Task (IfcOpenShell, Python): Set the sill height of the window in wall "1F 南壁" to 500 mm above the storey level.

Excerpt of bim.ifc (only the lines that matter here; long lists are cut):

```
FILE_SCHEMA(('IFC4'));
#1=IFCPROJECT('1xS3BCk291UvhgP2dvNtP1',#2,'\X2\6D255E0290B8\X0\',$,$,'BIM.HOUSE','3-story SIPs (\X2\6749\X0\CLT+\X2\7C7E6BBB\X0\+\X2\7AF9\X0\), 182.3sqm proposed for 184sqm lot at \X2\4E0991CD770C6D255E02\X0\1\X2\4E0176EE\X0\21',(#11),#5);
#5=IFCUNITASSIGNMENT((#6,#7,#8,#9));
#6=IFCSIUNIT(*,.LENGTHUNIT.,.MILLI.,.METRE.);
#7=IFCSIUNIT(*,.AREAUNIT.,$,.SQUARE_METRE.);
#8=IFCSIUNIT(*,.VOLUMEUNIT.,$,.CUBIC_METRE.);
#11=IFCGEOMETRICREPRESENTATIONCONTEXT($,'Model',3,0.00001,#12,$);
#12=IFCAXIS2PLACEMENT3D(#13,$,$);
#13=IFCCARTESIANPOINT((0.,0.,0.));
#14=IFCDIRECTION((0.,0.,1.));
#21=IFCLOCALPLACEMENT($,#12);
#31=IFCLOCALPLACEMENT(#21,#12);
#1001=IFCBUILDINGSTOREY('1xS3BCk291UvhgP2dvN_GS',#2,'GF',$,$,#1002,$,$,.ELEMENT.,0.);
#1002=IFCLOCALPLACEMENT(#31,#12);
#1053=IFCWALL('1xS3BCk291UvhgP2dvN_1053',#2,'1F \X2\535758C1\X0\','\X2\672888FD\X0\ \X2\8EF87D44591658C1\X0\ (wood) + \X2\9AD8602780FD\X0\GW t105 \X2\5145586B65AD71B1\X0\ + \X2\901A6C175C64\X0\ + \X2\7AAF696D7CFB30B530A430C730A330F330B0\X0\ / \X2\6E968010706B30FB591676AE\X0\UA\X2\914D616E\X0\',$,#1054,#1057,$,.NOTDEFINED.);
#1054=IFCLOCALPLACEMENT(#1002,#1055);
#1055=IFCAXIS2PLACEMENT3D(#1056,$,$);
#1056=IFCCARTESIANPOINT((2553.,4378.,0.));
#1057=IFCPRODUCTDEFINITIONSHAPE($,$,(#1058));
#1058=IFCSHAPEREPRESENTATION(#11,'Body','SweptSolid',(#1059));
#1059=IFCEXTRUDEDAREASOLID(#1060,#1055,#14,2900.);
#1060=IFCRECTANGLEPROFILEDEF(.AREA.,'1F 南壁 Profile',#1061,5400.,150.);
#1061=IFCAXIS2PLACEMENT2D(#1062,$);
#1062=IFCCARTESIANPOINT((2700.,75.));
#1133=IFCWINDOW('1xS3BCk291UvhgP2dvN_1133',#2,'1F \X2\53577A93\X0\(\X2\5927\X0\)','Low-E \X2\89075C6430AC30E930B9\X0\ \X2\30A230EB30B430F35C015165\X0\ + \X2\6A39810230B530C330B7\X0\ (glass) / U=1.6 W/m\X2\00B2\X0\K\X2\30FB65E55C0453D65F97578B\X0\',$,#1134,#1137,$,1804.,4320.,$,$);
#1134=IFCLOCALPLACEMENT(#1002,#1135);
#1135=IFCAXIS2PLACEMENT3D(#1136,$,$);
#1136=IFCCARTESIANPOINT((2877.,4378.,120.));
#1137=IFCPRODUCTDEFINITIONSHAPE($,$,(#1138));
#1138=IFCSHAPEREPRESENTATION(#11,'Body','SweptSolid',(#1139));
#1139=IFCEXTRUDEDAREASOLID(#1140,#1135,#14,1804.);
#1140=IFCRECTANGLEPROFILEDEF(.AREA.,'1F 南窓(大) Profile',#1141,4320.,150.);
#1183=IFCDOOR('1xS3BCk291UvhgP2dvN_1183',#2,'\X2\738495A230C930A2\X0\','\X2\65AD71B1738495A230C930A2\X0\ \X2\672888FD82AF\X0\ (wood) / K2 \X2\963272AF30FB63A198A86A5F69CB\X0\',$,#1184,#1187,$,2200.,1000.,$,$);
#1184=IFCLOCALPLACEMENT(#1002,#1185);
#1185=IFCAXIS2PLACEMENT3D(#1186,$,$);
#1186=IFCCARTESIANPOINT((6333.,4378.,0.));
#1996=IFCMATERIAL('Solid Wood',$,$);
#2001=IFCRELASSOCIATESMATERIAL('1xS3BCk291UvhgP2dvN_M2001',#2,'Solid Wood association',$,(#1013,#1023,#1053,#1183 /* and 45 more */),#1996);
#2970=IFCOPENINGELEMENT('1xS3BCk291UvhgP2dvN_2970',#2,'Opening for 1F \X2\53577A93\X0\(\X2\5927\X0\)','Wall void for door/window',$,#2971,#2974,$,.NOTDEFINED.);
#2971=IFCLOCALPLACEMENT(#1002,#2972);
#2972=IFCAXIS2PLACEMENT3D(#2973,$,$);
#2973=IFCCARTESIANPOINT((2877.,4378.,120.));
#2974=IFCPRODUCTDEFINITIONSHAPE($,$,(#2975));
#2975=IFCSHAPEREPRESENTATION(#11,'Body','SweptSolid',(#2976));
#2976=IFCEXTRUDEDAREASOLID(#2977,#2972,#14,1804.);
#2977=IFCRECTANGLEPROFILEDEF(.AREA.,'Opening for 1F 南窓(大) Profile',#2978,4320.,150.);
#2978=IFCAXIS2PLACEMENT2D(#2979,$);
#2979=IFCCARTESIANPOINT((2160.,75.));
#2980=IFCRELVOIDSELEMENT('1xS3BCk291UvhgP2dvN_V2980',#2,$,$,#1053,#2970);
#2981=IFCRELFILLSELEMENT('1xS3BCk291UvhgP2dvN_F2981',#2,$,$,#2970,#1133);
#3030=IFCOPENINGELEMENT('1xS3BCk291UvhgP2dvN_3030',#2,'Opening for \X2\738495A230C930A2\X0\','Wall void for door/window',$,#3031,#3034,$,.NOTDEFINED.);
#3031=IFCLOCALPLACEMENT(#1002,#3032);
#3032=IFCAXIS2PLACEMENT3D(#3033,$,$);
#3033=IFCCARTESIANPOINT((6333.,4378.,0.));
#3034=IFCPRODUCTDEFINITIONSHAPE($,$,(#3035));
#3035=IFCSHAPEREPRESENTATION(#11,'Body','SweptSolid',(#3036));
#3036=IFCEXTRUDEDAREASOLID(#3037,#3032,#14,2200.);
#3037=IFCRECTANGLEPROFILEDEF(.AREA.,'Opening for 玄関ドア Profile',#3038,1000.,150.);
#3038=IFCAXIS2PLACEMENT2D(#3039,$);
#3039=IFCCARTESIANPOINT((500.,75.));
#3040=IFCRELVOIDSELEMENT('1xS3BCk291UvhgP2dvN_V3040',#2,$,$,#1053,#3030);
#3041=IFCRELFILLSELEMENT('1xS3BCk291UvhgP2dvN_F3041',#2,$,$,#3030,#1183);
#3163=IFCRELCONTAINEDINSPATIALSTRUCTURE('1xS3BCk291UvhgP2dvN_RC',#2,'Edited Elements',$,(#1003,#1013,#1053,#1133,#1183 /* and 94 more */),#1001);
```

```python
import numpy as np
import ifcopenshell
import ifcopenshell.api.geometry
import ifcopenshell.geom
import ifcopenshell.util.element
import ifcopenshell.util.placement
import ifcopenshell.util.shape
import ifcopenshell.util.unit

model = ifcopenshell.open("bim.ifc")
unit_scale = ifcopenshell.util.unit.calculate_unit_scale(model)

window = model.by_guid("1xS3BCk291UvhgP2dvN_1133")
opening = window.FillsVoids[0].RelatingOpeningElement
storey = ifcopenshell.util.element.get_container(window, ifc_class="IfcBuildingStorey")
level = ifcopenshell.util.placement.get_local_placement(storey.ObjectPlacement)[2, 3]

# The opening's origin need not be at the sill, so measure its lowest point.
shape = ifcopenshell.geom.create_shape(ifcopenshell.geom.settings(), opening)
bottom = ifcopenshell.util.shape.get_shape_bottom_elevation(shape, shape.geometry) / unit_scale
dz = level + 0.5 / unit_scale - bottom

shift = np.array([0.0, 0.0, dz])
# The window is not placed relative to its opening, so move both.
for product in (opening, window):
    matrix = ifcopenshell.util.placement.get_local_placement(product.ObjectPlacement)
    matrix[:3, 3] += shift
    ifcopenshell.api.geometry.edit_object_placement(model, product=product, matrix=matrix, is_si=False)

print(f"moved by {dz * unit_scale:+.3f} m")

model.write("bim_updated.ifc")
```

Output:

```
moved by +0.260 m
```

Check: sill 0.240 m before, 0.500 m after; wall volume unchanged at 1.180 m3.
